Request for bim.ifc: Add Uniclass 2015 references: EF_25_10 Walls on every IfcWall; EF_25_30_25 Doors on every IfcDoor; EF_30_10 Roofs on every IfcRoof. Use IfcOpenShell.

First a look at what the model holds.

```python
import ifcopenshell

model = ifcopenshell.open("bim.ifc")
print(model.schema)
print("classifications:", [c.Name for c in model.by_type("IfcClassification")])
for ifc_class in ("IfcDoor", "IfcRoof", "IfcStair", "IfcWall", "IfcWindow"):
    print(ifc_class, len(model.by_type(ifc_class)))
```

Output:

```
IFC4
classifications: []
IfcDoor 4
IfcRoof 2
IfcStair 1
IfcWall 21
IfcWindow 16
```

```python
import ifcopenshell
import ifcopenshell.api.classification

model = ifcopenshell.open("bim.ifc")

system = ifcopenshell.api.classification.add_classification(model, classification="Uniclass 2015")

codes = {
    "IfcWall": ("EF_25_10", "Walls"),
    "IfcDoor": ("EF_25_30_25", "Doors"),
    "IfcRoof": ("EF_30_10", "Roofs"),
}
for ifc_class, (code, name) in codes.items():
    products = model.by_type(ifc_class)
    ifcopenshell.api.classification.add_reference(
        model, products=products, classification=system, identification=code, name=name
    )
    print(code, len(products))

model.write("bim-out.ifc")
```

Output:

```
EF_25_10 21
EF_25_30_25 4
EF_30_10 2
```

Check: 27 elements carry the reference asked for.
